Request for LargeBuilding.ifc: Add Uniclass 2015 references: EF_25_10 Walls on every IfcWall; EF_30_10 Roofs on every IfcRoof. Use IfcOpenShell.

First a look at what the model holds.

```python
import ifcopenshell

model = ifcopenshell.open("LargeBuilding.ifc")
print(model.schema)
print("classifications:", [c.Name for c in model.by_type("IfcClassification")])
for ifc_class in ("IfcDoor", "IfcRoof", "IfcStair", "IfcWall", "IfcWindow"):
    print(ifc_class, len(model.by_type(ifc_class)))
```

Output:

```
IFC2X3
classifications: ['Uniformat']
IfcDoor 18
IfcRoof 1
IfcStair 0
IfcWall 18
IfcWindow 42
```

```python
import ifcopenshell
import ifcopenshell.api.classification

model = ifcopenshell.open("LargeBuilding.ifc")

# IFC2X3 requires Source and Edition and has no link from the project to the system.
system = model.create_entity("IfcClassification", Source="NBS", Edition="2015", Name="Uniclass 2015")

codes = {
    "IfcWall": ("EF_25_10", "Walls"),
    "IfcRoof": ("EF_30_10", "Roofs"),
}
for ifc_class, (code, name) in codes.items():
    products = model.by_type(ifc_class)
    ifcopenshell.api.classification.add_reference(
        model, products=products, classification=system, identification=code, name=name
    )
    print(code, len(products))

model.write("LargeBuilding_edited.ifc")
```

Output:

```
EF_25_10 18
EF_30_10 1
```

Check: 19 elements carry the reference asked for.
